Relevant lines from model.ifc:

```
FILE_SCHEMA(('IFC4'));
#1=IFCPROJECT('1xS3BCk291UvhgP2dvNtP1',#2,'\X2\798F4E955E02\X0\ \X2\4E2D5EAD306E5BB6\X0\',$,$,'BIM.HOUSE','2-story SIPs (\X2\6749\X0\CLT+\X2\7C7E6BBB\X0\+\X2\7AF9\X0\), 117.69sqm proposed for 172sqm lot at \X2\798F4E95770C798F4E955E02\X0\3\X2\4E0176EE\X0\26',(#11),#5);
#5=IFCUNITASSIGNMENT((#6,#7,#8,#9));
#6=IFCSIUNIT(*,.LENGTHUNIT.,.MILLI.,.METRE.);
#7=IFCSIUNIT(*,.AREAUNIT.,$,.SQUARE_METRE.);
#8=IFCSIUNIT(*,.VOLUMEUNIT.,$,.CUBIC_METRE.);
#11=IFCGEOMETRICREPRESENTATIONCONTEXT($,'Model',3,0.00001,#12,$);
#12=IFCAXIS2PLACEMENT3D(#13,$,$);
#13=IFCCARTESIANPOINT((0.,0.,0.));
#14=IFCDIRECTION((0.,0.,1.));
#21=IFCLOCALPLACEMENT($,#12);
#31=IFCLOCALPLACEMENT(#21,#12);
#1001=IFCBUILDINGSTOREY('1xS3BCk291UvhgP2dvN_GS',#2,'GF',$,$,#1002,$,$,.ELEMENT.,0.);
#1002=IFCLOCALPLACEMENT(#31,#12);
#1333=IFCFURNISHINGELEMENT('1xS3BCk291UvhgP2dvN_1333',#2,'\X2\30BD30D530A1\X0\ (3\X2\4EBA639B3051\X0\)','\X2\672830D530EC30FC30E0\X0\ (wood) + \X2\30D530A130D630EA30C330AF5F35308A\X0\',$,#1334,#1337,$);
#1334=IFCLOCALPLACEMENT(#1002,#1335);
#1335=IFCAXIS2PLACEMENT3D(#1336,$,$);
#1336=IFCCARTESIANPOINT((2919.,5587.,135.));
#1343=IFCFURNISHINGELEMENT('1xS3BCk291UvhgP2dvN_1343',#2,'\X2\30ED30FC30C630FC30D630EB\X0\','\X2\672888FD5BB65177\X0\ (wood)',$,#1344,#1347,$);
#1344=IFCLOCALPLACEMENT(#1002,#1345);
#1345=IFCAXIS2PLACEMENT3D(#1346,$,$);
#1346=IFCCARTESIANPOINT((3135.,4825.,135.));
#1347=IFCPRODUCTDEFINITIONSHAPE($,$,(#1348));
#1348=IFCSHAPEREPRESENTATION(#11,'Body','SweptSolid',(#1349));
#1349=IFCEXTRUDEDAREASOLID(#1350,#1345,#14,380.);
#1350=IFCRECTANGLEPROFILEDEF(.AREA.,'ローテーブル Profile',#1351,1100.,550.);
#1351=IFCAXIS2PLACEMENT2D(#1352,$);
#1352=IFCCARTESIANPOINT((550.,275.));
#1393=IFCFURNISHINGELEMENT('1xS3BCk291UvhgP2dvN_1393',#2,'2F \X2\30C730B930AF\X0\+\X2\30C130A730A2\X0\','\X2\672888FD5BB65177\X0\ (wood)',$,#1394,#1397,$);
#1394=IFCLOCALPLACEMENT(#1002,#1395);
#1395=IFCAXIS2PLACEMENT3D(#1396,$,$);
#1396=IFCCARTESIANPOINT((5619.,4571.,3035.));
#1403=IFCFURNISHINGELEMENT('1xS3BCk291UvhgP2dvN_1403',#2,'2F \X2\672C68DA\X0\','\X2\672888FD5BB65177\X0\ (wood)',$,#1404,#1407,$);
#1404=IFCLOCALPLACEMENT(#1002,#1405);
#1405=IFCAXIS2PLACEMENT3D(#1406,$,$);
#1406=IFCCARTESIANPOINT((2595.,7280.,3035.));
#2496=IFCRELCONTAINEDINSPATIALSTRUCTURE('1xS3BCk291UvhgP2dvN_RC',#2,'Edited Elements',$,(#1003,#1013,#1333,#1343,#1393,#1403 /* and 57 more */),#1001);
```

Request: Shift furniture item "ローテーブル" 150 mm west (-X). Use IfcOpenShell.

```python
import ifcopenshell
import ifcopenshell.api.geometry
import ifcopenshell.util.placement
import ifcopenshell.util.unit

model = ifcopenshell.open("model.ifc")
unit_scale = ifcopenshell.util.unit.calculate_unit_scale(model)

item = model.by_guid("1xS3BCk291UvhgP2dvN_1343")
matrix = ifcopenshell.util.placement.get_local_placement(item.ObjectPlacement)
matrix[0, 3] -= 0.15 / unit_scale
ifcopenshell.api.geometry.edit_object_placement(model, product=item, matrix=matrix, is_si=False)

print(ifcopenshell.util.placement.get_local_placement(item.ObjectPlacement).round(3) + 0.0)

model.write("model_edited.ifc")
```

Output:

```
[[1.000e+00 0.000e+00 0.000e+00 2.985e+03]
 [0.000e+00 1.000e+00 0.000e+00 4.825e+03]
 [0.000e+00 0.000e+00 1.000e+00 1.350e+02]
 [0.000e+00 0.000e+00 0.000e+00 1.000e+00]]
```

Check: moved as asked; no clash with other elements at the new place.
